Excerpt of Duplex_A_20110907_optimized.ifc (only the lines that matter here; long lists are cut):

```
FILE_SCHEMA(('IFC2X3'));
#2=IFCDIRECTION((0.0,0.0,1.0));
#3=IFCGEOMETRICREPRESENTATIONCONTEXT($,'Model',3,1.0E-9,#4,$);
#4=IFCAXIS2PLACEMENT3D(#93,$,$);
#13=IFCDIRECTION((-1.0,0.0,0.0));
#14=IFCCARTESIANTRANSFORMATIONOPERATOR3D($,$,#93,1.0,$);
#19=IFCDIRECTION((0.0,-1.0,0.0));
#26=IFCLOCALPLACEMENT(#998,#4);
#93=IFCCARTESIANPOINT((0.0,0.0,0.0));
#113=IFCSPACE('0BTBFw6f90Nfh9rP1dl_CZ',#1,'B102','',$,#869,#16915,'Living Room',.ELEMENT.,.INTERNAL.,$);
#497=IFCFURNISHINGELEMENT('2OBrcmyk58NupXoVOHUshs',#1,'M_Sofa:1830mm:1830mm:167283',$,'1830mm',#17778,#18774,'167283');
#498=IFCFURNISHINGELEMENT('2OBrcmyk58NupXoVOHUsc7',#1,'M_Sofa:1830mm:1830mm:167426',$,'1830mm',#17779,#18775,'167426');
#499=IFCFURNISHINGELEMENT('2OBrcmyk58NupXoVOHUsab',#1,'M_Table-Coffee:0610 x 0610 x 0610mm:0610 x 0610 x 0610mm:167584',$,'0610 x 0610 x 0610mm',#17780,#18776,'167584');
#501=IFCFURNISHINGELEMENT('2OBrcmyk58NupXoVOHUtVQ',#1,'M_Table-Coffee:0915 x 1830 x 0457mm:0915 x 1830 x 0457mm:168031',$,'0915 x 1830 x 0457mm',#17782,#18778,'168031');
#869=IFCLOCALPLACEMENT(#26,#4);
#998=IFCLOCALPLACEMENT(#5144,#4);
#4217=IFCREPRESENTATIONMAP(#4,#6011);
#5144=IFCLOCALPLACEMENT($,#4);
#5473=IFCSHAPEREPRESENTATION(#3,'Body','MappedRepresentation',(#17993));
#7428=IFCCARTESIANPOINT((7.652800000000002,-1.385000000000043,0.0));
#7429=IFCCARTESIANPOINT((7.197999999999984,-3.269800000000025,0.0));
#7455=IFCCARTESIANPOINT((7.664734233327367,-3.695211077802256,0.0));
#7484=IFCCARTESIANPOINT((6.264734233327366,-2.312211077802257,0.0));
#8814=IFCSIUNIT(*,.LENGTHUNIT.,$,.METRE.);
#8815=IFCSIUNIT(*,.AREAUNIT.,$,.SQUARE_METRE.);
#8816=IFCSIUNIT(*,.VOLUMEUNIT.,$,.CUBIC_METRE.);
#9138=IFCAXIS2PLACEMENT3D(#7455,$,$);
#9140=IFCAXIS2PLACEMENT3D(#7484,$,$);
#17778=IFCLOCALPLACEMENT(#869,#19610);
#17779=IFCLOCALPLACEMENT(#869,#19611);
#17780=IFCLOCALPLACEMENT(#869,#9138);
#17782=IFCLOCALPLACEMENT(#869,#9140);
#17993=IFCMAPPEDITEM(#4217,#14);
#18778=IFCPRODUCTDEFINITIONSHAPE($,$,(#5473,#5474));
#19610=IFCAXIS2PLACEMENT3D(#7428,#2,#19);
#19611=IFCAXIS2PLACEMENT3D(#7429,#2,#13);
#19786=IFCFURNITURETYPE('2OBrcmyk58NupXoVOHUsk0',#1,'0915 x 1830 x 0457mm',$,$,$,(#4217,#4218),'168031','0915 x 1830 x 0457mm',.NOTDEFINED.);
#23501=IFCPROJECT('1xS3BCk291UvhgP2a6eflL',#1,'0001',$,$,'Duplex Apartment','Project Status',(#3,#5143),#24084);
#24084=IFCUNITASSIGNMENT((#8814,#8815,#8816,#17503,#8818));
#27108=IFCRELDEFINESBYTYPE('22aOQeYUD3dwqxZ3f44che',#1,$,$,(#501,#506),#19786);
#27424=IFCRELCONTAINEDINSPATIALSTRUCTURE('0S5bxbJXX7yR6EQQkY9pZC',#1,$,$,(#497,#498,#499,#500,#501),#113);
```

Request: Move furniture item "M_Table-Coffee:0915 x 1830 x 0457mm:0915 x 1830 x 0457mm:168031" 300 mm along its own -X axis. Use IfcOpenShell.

```python
import ifcopenshell
import ifcopenshell.api.geometry
import ifcopenshell.util.placement
import ifcopenshell.util.unit

model = ifcopenshell.open("Duplex_A_20110907_optimized.ifc")
unit_scale = ifcopenshell.util.unit.calculate_unit_scale(model)

item = model.by_guid("2OBrcmyk58NupXoVOHUtVQ")
matrix = ifcopenshell.util.placement.get_local_placement(item.ObjectPlacement)
matrix[:3, 3] -= matrix[:3, 0] * 0.3 / unit_scale
ifcopenshell.api.geometry.edit_object_placement(model, product=item, matrix=matrix, is_si=False)

print(ifcopenshell.util.placement.get_local_placement(item.ObjectPlacement).round(3) + 0.0)

model.write("Duplex_A_20110907_optimized-out.ifc")
```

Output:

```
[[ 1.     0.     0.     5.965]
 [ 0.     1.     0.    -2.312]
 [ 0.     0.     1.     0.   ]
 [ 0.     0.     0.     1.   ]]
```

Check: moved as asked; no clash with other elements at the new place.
